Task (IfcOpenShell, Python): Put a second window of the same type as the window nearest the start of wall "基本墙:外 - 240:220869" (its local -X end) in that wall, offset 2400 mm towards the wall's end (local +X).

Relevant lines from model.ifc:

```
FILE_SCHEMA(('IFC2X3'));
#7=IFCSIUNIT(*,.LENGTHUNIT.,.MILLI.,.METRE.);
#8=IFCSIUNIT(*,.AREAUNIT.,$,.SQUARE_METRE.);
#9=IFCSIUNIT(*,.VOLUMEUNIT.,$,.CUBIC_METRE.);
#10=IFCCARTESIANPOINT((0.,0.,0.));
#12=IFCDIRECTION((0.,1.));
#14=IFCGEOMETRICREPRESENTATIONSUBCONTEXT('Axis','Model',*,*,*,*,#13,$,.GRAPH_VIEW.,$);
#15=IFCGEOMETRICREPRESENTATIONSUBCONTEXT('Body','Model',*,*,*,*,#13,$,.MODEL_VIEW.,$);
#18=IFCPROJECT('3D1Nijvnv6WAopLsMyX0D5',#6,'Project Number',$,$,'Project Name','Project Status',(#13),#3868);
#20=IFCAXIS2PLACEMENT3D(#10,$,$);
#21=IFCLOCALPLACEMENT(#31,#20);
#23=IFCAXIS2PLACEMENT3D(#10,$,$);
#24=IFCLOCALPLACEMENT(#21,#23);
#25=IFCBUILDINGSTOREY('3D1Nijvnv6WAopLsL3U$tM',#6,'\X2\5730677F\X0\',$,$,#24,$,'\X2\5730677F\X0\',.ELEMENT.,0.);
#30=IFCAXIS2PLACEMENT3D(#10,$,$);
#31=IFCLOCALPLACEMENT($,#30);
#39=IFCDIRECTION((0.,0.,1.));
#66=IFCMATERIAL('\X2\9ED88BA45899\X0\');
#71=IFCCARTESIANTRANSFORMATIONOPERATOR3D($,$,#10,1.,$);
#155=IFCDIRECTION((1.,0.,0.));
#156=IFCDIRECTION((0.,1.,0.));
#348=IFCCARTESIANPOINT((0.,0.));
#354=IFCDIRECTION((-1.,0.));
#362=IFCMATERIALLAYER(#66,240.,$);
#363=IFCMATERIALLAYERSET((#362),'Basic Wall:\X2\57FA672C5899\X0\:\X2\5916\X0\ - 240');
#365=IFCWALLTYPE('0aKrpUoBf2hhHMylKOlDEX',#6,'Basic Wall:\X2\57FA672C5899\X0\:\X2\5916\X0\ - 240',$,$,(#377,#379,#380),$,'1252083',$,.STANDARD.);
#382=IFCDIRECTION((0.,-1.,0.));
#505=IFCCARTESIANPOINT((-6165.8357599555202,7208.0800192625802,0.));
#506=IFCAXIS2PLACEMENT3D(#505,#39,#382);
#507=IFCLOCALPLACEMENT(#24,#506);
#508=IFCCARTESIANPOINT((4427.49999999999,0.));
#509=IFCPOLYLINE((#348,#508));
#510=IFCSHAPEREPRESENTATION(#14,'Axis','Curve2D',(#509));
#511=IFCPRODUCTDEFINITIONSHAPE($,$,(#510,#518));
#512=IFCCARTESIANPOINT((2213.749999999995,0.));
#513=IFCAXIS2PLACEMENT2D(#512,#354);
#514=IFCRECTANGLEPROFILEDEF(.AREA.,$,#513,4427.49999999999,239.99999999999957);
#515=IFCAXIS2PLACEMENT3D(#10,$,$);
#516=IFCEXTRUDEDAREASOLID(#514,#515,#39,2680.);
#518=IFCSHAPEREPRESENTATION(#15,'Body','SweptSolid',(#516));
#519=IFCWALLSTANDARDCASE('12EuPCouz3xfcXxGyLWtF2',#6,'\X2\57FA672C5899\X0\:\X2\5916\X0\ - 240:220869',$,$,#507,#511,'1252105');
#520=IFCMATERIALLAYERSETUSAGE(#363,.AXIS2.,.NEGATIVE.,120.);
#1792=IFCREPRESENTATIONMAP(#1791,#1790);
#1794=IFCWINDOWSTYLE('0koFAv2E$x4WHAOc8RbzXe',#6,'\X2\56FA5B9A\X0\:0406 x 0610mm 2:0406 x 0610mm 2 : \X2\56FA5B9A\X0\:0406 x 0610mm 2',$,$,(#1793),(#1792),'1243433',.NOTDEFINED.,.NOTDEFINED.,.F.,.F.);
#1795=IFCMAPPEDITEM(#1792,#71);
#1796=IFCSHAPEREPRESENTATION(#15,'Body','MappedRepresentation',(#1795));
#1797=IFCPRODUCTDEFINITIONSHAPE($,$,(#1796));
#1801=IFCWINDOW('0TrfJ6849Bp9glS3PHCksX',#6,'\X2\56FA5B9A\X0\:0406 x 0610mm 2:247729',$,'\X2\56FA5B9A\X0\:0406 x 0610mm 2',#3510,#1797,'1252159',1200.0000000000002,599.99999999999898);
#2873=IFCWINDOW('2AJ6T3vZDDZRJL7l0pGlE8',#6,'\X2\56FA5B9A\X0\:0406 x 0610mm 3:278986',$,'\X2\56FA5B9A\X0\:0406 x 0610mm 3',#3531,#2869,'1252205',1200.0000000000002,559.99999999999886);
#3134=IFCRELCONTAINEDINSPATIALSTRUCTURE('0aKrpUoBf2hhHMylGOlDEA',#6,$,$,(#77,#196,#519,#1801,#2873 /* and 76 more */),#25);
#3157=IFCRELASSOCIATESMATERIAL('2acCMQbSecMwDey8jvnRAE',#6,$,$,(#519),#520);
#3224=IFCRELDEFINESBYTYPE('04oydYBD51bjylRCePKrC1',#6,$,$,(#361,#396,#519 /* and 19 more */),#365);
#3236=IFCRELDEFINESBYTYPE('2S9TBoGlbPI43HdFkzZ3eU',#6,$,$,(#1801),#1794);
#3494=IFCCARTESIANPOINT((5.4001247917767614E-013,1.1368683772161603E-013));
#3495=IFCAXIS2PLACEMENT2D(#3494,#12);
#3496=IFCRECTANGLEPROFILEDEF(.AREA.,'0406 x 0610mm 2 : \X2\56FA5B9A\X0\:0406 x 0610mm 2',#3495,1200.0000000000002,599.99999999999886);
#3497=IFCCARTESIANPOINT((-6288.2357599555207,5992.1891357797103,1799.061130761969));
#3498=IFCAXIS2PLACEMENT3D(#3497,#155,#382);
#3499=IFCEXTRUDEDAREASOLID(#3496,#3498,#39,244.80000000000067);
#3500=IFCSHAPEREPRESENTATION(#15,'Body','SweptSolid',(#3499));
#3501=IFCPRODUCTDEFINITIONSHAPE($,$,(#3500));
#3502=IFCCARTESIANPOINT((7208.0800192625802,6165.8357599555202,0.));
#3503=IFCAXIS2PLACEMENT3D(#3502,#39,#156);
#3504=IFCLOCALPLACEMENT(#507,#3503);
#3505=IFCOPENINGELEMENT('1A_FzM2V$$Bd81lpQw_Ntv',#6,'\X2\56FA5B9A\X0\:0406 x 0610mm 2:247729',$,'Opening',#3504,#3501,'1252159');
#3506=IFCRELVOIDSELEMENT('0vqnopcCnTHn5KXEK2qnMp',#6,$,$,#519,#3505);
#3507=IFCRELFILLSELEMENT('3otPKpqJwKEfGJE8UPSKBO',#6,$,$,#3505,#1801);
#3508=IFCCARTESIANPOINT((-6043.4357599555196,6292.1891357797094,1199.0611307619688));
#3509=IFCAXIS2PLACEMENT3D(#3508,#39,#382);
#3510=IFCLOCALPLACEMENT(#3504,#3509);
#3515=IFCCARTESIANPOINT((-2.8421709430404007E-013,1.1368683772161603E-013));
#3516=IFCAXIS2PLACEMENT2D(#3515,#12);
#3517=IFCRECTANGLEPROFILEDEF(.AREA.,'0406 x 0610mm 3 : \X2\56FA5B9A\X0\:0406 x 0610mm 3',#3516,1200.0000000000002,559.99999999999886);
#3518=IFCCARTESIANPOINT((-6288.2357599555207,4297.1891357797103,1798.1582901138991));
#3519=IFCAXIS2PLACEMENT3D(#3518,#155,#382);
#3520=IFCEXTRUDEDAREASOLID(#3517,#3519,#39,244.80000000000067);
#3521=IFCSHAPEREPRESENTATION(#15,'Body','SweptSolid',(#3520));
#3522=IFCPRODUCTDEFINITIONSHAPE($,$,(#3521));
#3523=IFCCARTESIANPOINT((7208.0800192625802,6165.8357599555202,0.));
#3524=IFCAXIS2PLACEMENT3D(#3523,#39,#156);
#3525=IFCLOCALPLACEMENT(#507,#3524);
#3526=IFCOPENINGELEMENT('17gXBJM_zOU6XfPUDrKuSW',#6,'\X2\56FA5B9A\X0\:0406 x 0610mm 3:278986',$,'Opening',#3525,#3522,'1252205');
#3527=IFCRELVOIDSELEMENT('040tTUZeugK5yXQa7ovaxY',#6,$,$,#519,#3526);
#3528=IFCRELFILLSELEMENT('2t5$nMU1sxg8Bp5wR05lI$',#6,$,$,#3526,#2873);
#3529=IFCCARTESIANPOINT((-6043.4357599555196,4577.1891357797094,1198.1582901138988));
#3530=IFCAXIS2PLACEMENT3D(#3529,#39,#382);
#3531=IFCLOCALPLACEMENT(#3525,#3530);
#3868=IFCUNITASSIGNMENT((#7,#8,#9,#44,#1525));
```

```python
import ifcopenshell
import ifcopenshell.api.feature
import ifcopenshell.api.geometry
import ifcopenshell.api.root
import ifcopenshell.geom
import ifcopenshell.util.element
import ifcopenshell.util.placement
import ifcopenshell.util.shape
import ifcopenshell.util.unit

model = ifcopenshell.open("model.ifc")
unit_scale = ifcopenshell.util.unit.calculate_unit_scale(model)
settings = ifcopenshell.geom.settings()


def volume(element):
    """Net volume in cubic metres, openings subtracted."""
    shape = ifcopenshell.geom.create_shape(settings, element)
    return ifcopenshell.util.shape.get_volume(shape.geometry)


def reuse_history(source, copy):
    """copy_class also copies each property set's owner history, people and application; keep the originals."""
    for rel in copy.IsDefinedBy:
        if rel.is_a("IfcRelDefinesByProperties") and (history := rel.RelatingPropertyDefinition.OwnerHistory):
            rel.RelatingPropertyDefinition.OwnerHistory = source.OwnerHistory
            ifcopenshell.util.element.remove_deep2(model, history)


window = model.by_id(1801)
opening = window.FillsVoids[0].RelatingOpeningElement
wall = opening.VoidsElements[0].RelatingBuildingElement
before = volume(wall)
shift = ifcopenshell.util.placement.get_local_placement(wall.ObjectPlacement)[:3, 0] * 2.4 / unit_scale

# copy_class copies the void relationship, type, container and properties, but no geometry.
new_opening = ifcopenshell.api.root.copy_class(model, product=opening)
new_opening.Representation = ifcopenshell.util.element.copy_deep(
    model, opening.Representation, exclude=["IfcGeometricRepresentationContext", "IfcRepresentationMap"]
)
new_opening.Name = "固定:0406 x 0610mm 2"
new_opening.Tag = None
new_window = ifcopenshell.api.root.copy_class(model, product=window)
new_window.Representation = ifcopenshell.util.element.copy_deep(
    model, window.Representation, exclude=["IfcGeometricRepresentationContext", "IfcRepresentationMap"]
)
new_window.Name = "固定:0406 x 0610mm 2"
new_window.Tag = None
reuse_history(window, new_window)
fills = ifcopenshell.api.feature.add_filling(model, opening=new_opening, element=new_window)
fills.OwnerHistory = new_window.OwnerHistory  # required in IFC2X3

for old, new in ((opening, new_opening), (window, new_window)):
    matrix = ifcopenshell.util.placement.get_local_placement(old.ObjectPlacement)
    matrix[:3, 3] += shift
    ifcopenshell.api.geometry.edit_object_placement(model, product=new, matrix=matrix, is_si=False)

after = volume(wall)

print(f"wall volume {before:.3f} -> {after:.3f} m3")

model.write("model_v2.ifc")
```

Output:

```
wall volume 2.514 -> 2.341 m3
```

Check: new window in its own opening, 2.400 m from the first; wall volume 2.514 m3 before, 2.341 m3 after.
